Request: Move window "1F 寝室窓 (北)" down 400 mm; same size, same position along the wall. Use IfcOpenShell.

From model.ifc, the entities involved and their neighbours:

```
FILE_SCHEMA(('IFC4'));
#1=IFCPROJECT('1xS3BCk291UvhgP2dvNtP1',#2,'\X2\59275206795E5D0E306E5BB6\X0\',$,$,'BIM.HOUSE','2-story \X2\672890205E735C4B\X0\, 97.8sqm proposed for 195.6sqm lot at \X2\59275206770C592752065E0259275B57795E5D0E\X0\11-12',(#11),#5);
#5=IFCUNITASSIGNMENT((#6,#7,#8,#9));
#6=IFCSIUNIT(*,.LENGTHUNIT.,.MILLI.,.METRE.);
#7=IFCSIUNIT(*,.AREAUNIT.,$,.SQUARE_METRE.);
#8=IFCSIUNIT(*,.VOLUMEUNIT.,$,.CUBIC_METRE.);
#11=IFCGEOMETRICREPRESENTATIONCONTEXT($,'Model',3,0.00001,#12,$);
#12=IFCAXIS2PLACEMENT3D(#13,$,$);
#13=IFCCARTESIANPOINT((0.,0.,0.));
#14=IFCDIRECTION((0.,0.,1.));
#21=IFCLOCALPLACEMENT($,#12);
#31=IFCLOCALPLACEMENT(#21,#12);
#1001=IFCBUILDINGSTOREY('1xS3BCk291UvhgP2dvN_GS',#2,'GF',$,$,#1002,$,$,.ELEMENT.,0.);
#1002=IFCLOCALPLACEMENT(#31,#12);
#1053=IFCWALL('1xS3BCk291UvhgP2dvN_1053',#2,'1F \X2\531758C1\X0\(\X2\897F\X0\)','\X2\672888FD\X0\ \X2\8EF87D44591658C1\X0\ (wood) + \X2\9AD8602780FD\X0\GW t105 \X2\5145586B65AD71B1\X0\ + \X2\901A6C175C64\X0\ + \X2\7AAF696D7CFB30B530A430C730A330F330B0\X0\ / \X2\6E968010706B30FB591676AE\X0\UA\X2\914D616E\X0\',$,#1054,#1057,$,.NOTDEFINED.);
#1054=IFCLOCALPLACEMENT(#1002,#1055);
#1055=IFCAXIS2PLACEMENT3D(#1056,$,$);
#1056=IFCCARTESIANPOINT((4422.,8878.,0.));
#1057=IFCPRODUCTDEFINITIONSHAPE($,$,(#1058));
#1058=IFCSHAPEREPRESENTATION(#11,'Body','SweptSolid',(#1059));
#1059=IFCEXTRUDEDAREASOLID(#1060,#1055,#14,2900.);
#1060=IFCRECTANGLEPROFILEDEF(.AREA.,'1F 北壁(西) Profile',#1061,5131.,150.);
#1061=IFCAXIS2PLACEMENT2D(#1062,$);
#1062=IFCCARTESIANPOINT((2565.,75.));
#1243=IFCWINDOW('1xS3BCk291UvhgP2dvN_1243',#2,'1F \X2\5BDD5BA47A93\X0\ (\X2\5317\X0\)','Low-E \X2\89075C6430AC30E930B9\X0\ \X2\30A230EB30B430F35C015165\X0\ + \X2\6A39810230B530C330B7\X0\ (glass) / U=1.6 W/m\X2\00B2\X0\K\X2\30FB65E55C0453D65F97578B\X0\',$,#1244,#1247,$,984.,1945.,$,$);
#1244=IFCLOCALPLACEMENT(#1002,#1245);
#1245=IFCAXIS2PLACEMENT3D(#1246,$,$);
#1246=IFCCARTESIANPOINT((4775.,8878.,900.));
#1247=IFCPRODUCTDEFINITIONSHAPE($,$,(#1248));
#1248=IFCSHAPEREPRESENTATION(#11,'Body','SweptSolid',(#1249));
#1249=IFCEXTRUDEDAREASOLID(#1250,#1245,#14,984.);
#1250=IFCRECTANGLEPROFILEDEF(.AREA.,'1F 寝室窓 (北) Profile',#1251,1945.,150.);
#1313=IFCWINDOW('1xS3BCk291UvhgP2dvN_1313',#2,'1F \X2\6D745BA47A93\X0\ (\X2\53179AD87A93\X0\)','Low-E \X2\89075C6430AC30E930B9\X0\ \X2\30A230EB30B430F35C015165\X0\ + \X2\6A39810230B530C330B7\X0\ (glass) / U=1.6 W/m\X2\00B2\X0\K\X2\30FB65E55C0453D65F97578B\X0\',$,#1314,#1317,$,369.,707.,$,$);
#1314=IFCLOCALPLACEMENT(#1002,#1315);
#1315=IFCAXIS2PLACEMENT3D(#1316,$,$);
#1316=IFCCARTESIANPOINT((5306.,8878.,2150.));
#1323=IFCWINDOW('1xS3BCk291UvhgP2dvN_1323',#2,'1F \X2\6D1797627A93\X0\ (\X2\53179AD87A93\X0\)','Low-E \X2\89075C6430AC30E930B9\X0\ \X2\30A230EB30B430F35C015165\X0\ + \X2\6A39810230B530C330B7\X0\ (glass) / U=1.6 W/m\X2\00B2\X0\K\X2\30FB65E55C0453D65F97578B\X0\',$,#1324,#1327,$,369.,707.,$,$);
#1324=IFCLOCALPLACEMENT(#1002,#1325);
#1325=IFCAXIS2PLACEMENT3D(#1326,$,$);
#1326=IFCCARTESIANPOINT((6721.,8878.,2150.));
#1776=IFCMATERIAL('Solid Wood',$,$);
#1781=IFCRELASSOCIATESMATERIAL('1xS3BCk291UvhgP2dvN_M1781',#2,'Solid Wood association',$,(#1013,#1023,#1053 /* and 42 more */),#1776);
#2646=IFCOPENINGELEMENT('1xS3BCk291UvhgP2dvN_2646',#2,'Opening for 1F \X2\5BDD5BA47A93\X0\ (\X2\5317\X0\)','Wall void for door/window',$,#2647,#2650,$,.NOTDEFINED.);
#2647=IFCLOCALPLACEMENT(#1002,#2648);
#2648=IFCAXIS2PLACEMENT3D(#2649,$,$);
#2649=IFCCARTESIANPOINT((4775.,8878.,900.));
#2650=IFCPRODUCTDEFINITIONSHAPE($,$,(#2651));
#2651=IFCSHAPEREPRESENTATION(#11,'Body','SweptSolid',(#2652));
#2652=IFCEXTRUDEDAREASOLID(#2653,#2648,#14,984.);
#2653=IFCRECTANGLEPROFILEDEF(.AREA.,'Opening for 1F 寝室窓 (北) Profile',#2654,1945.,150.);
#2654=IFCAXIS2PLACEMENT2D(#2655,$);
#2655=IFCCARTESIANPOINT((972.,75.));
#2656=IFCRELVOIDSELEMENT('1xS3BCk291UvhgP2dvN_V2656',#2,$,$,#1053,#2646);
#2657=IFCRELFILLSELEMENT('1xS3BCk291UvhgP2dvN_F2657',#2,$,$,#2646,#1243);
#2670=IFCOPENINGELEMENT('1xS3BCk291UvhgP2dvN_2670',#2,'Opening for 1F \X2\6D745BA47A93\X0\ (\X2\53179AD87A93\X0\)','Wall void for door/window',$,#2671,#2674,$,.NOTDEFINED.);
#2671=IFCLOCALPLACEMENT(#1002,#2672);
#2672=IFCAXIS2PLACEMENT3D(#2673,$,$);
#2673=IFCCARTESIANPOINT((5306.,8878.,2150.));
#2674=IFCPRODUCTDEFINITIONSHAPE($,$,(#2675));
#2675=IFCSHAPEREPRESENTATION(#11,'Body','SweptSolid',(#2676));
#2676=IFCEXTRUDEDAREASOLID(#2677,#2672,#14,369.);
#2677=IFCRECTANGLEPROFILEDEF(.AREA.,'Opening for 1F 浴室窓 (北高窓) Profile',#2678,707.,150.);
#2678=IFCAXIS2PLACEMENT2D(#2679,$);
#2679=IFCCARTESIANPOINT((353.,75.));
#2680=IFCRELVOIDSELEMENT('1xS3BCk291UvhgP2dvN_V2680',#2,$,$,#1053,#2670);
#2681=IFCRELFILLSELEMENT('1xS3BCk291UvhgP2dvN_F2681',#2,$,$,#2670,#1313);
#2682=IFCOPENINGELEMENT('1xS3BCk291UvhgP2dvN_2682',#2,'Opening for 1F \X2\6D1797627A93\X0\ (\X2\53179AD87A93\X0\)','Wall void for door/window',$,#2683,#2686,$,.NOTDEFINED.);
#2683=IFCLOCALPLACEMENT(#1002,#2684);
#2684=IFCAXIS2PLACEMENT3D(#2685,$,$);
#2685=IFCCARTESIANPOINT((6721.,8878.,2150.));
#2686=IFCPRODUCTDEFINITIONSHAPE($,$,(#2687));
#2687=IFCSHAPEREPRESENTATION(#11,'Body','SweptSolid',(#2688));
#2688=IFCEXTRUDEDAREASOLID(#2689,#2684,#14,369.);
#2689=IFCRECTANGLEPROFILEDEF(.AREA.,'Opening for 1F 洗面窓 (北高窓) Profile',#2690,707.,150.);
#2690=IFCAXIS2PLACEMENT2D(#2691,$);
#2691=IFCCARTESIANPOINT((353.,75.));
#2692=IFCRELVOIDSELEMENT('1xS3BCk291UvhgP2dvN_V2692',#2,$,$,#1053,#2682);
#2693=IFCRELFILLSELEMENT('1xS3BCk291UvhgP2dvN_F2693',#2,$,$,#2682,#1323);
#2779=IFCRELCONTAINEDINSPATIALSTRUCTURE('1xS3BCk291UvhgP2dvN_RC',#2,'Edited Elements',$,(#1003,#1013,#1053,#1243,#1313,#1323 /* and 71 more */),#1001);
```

```python
import numpy as np
import ifcopenshell
import ifcopenshell.api.geometry
import ifcopenshell.util.placement
import ifcopenshell.util.unit

model = ifcopenshell.open("model.ifc")
unit_scale = ifcopenshell.util.unit.calculate_unit_scale(model)

window = model.by_guid("1xS3BCk291UvhgP2dvN_1243")
opening = window.FillsVoids[0].RelatingOpeningElement
dz = -400.0

shift = np.array([0.0, 0.0, dz])
# The window is not placed relative to its opening, so move both.
for product in (opening, window):
    matrix = ifcopenshell.util.placement.get_local_placement(product.ObjectPlacement)
    matrix[:3, 3] += shift
    ifcopenshell.api.geometry.edit_object_placement(model, product=product, matrix=matrix, is_si=False)

print(f"moved by {dz * unit_scale:+.3f} m")

model.write("model_edited.ifc")
```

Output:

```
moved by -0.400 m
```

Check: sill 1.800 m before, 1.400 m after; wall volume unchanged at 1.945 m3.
